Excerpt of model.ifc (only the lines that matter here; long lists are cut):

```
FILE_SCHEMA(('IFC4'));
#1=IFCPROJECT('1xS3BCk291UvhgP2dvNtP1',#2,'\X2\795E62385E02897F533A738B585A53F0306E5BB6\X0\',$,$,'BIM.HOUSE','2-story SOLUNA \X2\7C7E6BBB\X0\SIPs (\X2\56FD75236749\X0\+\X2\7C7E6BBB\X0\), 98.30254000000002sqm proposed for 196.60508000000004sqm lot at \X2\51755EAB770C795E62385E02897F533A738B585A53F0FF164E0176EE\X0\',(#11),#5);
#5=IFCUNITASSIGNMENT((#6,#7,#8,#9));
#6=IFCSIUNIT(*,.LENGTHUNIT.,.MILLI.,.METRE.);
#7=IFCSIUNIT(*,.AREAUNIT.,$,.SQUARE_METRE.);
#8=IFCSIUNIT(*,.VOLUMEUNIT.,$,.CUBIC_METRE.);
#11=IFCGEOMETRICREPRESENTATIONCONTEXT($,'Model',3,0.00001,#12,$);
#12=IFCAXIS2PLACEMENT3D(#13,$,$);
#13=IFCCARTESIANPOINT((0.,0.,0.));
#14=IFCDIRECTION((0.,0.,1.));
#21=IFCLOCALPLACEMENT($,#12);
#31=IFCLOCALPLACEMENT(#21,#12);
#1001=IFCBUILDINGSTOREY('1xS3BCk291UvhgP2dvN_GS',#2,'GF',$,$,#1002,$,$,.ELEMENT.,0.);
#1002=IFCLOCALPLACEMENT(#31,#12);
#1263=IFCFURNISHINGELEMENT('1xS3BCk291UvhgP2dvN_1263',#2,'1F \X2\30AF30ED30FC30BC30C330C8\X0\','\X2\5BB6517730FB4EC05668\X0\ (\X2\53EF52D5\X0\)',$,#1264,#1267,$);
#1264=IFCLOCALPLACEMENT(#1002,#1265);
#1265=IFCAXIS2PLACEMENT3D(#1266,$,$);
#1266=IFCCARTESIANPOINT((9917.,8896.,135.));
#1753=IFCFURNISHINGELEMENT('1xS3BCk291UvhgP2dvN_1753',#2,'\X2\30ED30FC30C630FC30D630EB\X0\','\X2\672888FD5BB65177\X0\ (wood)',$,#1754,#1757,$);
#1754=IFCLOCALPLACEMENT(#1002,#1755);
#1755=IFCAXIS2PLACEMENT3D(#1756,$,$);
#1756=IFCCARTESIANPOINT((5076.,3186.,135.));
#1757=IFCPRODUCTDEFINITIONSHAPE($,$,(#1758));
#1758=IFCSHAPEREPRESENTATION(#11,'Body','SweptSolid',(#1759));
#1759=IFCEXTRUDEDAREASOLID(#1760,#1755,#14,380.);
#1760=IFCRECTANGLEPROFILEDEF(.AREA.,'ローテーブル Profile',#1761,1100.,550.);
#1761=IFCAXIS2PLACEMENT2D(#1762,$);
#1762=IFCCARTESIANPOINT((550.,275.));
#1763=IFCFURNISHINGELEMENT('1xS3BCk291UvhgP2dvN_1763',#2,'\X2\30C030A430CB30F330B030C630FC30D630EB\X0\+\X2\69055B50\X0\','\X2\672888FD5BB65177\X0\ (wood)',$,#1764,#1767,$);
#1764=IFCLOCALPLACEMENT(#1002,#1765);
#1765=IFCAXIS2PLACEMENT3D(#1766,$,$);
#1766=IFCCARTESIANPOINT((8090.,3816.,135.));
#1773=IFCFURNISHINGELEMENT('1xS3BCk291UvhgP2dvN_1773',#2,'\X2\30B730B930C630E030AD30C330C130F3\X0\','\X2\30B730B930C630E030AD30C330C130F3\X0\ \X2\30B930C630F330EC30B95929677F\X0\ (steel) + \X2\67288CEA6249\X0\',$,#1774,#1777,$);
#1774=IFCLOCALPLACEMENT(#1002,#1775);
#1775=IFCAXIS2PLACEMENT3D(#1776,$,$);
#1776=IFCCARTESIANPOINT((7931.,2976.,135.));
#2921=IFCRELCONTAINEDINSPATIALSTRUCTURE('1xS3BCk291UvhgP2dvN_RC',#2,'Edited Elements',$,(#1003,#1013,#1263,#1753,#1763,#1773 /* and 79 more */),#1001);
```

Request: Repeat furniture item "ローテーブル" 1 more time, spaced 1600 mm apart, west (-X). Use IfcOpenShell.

```python
import numpy as np
import ifcopenshell
import ifcopenshell.api.geometry
import ifcopenshell.api.root
import ifcopenshell.util.element
import ifcopenshell.util.placement
import ifcopenshell.util.unit

model = ifcopenshell.open("model.ifc")
unit_scale = ifcopenshell.util.unit.calculate_unit_scale(model)


def reuse_history(source, copy):
    """copy_class also copies each property set's owner history, people and application; keep the originals."""
    for rel in copy.IsDefinedBy:
        if rel.is_a("IfcRelDefinesByProperties") and (history := rel.RelatingPropertyDefinition.OwnerHistory):
            rel.RelatingPropertyDefinition.OwnerHistory = source.OwnerHistory
            ifcopenshell.util.element.remove_deep2(model, history)


source = model.by_id(1753)
base = ifcopenshell.util.placement.get_local_placement(source.ObjectPlacement)
step = np.array([-1.0, 0.0, 0.0]) * 1.6 / unit_scale

for i in range(1, 2):
    copy = ifcopenshell.api.root.copy_class(model, product=source)
    copy.Representation = ifcopenshell.util.element.copy_deep(
        model, source.Representation, exclude=["IfcGeometricRepresentationContext", "IfcRepresentationMap"]
    )
    reuse_history(source, copy)
    matrix = base.copy()
    matrix[:3, 3] += i * step
    print("added at", matrix[:3, 3].round(3) + 0.0)
    ifcopenshell.api.geometry.edit_object_placement(model, product=copy, matrix=matrix, is_si=False)

model.write("model-out.ifc")
```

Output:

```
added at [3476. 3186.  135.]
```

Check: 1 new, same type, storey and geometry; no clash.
